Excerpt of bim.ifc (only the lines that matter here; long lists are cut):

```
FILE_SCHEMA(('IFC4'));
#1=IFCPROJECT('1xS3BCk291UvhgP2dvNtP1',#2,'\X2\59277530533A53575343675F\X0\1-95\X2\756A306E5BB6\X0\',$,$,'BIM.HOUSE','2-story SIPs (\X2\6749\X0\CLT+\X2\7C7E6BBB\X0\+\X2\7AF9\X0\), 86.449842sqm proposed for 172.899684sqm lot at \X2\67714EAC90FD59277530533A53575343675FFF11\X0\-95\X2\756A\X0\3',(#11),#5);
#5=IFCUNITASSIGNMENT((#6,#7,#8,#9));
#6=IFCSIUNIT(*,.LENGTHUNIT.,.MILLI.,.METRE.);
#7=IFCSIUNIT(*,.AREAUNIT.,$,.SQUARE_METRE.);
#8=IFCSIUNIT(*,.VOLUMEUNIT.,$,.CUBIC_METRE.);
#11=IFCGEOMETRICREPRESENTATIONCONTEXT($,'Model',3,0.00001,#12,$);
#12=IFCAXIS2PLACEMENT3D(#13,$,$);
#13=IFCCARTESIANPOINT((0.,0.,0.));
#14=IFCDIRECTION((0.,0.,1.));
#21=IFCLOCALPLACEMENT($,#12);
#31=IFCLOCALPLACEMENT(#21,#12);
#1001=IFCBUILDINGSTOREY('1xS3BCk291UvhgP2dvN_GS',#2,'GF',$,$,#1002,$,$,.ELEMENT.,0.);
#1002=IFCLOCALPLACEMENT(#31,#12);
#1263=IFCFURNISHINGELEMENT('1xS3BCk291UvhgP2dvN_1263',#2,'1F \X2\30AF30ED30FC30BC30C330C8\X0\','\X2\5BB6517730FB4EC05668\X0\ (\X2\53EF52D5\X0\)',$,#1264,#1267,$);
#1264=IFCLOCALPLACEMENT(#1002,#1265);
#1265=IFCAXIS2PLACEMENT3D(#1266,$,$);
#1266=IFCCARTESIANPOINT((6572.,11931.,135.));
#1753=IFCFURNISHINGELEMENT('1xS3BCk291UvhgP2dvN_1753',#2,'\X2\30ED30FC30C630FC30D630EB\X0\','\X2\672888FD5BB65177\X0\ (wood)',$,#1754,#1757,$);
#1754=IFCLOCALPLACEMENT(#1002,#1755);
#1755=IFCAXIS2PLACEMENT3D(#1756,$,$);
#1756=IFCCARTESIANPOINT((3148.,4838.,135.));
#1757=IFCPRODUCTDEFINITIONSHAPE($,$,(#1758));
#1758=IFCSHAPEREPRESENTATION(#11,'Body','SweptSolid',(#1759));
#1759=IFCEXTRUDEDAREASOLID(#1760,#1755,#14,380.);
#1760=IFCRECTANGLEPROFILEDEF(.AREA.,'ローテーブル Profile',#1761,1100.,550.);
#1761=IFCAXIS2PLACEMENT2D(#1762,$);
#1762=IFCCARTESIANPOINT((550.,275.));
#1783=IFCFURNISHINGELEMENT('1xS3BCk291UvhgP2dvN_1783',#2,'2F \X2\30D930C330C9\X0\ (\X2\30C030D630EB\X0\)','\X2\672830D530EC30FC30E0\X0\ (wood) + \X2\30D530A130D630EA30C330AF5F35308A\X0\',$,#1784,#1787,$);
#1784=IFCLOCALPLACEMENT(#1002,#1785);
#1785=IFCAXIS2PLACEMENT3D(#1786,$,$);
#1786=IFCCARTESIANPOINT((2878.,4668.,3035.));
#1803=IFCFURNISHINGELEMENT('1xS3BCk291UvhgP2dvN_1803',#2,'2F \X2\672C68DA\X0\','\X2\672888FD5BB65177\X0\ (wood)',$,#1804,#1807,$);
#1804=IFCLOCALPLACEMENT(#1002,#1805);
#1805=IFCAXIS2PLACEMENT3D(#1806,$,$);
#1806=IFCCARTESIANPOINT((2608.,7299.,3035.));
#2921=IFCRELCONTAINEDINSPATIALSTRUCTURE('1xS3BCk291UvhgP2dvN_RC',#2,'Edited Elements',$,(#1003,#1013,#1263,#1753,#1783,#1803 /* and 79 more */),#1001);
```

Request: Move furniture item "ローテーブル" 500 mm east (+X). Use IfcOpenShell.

```python
import ifcopenshell
import ifcopenshell.api.geometry
import ifcopenshell.util.placement
import ifcopenshell.util.unit

model = ifcopenshell.open("bim.ifc")
unit_scale = ifcopenshell.util.unit.calculate_unit_scale(model)

item = model.by_guid("1xS3BCk291UvhgP2dvN_1753")
matrix = ifcopenshell.util.placement.get_local_placement(item.ObjectPlacement)
matrix[0, 3] += 0.5 / unit_scale
ifcopenshell.api.geometry.edit_object_placement(model, product=item, matrix=matrix, is_si=False)

print(ifcopenshell.util.placement.get_local_placement(item.ObjectPlacement).round(3) + 0.0)

model.write("bim_updated.ifc")
```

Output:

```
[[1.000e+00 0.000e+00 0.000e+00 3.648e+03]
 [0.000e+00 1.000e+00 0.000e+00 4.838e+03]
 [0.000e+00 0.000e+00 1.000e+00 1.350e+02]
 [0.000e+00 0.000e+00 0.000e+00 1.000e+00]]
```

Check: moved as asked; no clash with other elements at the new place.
